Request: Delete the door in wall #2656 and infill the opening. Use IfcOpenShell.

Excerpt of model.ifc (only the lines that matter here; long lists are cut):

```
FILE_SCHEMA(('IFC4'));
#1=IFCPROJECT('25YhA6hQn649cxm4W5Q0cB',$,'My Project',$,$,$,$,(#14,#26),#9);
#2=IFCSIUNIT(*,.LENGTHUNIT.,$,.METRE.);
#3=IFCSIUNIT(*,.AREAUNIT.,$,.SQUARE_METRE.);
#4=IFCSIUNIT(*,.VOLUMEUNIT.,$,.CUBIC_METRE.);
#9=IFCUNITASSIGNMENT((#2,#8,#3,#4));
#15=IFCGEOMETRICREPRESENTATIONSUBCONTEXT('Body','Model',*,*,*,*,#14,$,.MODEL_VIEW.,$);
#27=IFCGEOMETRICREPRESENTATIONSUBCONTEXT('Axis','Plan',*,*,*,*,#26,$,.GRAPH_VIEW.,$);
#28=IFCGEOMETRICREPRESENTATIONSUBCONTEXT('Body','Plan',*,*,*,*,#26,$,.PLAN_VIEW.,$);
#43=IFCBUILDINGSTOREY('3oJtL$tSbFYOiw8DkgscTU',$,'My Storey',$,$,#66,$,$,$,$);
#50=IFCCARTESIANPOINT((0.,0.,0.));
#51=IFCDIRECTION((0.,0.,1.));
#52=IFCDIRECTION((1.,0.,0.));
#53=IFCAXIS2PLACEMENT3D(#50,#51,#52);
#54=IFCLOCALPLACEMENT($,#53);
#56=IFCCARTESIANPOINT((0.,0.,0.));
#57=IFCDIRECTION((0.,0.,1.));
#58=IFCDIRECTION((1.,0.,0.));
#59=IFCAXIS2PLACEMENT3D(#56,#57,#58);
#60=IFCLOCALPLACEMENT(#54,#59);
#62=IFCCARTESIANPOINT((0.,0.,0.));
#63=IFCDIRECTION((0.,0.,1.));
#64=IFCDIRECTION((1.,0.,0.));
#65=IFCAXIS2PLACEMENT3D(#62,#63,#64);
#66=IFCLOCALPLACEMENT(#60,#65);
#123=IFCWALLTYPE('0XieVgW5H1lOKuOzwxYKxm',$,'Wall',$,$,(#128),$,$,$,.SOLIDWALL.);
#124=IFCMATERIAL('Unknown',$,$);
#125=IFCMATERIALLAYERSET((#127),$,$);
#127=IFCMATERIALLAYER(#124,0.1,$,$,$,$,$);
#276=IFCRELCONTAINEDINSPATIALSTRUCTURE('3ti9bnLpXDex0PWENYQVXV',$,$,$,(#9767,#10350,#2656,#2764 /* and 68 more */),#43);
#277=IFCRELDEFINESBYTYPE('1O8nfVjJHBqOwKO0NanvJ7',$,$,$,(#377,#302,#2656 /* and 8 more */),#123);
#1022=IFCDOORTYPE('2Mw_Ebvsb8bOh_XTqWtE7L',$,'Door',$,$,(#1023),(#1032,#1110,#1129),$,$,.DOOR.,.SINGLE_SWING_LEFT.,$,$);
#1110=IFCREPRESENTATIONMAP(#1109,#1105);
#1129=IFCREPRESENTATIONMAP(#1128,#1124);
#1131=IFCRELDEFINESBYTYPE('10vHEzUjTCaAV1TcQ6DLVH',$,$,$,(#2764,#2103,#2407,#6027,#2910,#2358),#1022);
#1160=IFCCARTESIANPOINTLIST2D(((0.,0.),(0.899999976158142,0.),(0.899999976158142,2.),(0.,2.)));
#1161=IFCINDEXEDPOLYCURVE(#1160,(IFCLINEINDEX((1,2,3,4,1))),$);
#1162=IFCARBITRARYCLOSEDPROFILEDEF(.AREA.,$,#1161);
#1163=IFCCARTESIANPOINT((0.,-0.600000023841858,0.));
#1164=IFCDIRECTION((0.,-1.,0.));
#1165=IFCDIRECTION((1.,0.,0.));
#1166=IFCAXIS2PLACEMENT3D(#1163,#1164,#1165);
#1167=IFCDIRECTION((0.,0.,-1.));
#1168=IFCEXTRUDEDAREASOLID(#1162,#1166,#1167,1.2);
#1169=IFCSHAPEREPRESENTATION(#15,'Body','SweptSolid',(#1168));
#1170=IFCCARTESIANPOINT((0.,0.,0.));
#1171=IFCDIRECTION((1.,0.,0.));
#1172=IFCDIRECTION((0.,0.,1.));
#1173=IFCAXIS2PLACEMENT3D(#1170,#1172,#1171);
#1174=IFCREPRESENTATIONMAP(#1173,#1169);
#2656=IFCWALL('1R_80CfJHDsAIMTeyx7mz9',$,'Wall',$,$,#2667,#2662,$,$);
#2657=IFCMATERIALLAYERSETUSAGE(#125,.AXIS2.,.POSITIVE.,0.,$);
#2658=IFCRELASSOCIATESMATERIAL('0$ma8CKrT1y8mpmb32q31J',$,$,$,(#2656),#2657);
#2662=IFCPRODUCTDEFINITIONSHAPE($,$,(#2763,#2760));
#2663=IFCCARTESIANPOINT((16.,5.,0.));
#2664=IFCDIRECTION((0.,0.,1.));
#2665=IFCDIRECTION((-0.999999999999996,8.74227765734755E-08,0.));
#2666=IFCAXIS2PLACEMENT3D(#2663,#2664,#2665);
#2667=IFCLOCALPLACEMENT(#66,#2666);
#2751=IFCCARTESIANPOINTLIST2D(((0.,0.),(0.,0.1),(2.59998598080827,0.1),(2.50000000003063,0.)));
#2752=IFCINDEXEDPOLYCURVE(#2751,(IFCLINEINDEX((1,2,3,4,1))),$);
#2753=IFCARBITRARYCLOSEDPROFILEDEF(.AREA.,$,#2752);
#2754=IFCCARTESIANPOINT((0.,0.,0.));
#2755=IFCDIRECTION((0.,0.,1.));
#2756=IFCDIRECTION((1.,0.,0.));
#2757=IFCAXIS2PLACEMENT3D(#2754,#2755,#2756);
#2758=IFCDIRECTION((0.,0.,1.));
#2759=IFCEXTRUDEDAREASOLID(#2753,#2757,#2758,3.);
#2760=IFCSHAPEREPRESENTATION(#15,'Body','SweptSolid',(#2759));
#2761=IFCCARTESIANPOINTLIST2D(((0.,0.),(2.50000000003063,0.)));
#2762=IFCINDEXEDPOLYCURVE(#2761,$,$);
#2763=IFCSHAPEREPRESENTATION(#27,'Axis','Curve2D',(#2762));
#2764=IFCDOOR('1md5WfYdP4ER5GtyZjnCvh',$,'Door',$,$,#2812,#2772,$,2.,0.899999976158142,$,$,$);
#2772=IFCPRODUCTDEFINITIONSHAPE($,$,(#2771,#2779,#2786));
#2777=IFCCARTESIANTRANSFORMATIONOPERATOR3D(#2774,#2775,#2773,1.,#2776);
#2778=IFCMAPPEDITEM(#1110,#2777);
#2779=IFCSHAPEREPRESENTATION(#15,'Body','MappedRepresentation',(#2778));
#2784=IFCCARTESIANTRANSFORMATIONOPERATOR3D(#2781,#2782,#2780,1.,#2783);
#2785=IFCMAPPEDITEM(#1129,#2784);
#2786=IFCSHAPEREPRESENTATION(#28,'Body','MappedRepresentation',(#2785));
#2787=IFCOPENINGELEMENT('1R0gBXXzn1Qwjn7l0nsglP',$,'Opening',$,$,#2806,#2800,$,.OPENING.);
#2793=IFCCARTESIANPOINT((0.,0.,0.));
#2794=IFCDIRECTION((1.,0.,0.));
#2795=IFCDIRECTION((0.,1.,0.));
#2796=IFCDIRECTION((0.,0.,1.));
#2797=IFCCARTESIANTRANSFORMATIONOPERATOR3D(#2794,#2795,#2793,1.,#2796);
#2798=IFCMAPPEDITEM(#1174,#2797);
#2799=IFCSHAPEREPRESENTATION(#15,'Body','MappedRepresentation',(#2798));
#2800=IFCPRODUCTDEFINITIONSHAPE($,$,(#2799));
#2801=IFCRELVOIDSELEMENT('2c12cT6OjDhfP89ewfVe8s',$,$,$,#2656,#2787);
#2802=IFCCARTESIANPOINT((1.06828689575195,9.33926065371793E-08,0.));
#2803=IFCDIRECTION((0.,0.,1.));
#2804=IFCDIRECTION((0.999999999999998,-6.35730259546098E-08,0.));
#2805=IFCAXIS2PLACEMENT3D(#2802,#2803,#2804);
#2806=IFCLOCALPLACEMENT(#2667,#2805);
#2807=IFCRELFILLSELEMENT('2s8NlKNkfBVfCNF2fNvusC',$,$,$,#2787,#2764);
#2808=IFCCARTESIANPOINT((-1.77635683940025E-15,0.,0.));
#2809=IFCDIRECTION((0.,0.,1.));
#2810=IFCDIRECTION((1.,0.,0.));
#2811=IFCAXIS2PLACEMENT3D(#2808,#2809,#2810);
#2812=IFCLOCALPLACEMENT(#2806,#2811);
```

```python
import ifcopenshell
import ifcopenshell.api.feature
import ifcopenshell.api.root
import ifcopenshell.geom
import ifcopenshell.util.shape

model = ifcopenshell.open("model.ifc")
settings = ifcopenshell.geom.settings()


def volume(element):
    """Net volume in cubic metres, openings subtracted."""
    shape = ifcopenshell.geom.create_shape(settings, element)
    return ifcopenshell.util.shape.get_volume(shape.geometry)


door = model.by_guid("1md5WfYdP4ER5GtyZjnCvh")
opening = door.FillsVoids[0].RelatingOpeningElement
wall = opening.VoidsElements[0].RelatingBuildingElement
before = volume(wall)

ifcopenshell.api.root.remove_product(model, product=door)
ifcopenshell.api.feature.remove_feature(model, feature=opening)

after = volume(wall)

print(f"wall volume {before:.3f} -> {after:.3f} m3")

model.write("model_v2.ifc")
```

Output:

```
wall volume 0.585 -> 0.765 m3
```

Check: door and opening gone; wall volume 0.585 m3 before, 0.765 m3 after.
